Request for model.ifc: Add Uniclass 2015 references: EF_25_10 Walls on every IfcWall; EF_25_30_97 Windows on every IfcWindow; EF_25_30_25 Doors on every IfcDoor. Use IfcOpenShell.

First a look at what the model holds.

```python
import ifcopenshell

model = ifcopenshell.open("model.ifc")
print(model.schema)
print("classifications:", [c.Name for c in model.by_type("IfcClassification")])
for ifc_class in ("IfcDoor", "IfcRoof", "IfcStair", "IfcWall", "IfcWindow"):
    print(ifc_class, len(model.by_type(ifc_class)))
```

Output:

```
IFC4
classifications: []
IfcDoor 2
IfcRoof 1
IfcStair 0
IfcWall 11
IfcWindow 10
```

```python
import ifcopenshell
import ifcopenshell.api.classification

model = ifcopenshell.open("model.ifc")

system = ifcopenshell.api.classification.add_classification(model, classification="Uniclass 2015")

codes = {
    "IfcWall": ("EF_25_10", "Walls"),
    "IfcWindow": ("EF_25_30_97", "Windows"),
    "IfcDoor": ("EF_25_30_25", "Doors"),
}
for ifc_class, (code, name) in codes.items():
    products = model.by_type(ifc_class)
    ifcopenshell.api.classification.add_reference(
        model, products=products, classification=system, identification=code, name=name
    )
    print(code, len(products))

model.write("model_v2.ifc")
```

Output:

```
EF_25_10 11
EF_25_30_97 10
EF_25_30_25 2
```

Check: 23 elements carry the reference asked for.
